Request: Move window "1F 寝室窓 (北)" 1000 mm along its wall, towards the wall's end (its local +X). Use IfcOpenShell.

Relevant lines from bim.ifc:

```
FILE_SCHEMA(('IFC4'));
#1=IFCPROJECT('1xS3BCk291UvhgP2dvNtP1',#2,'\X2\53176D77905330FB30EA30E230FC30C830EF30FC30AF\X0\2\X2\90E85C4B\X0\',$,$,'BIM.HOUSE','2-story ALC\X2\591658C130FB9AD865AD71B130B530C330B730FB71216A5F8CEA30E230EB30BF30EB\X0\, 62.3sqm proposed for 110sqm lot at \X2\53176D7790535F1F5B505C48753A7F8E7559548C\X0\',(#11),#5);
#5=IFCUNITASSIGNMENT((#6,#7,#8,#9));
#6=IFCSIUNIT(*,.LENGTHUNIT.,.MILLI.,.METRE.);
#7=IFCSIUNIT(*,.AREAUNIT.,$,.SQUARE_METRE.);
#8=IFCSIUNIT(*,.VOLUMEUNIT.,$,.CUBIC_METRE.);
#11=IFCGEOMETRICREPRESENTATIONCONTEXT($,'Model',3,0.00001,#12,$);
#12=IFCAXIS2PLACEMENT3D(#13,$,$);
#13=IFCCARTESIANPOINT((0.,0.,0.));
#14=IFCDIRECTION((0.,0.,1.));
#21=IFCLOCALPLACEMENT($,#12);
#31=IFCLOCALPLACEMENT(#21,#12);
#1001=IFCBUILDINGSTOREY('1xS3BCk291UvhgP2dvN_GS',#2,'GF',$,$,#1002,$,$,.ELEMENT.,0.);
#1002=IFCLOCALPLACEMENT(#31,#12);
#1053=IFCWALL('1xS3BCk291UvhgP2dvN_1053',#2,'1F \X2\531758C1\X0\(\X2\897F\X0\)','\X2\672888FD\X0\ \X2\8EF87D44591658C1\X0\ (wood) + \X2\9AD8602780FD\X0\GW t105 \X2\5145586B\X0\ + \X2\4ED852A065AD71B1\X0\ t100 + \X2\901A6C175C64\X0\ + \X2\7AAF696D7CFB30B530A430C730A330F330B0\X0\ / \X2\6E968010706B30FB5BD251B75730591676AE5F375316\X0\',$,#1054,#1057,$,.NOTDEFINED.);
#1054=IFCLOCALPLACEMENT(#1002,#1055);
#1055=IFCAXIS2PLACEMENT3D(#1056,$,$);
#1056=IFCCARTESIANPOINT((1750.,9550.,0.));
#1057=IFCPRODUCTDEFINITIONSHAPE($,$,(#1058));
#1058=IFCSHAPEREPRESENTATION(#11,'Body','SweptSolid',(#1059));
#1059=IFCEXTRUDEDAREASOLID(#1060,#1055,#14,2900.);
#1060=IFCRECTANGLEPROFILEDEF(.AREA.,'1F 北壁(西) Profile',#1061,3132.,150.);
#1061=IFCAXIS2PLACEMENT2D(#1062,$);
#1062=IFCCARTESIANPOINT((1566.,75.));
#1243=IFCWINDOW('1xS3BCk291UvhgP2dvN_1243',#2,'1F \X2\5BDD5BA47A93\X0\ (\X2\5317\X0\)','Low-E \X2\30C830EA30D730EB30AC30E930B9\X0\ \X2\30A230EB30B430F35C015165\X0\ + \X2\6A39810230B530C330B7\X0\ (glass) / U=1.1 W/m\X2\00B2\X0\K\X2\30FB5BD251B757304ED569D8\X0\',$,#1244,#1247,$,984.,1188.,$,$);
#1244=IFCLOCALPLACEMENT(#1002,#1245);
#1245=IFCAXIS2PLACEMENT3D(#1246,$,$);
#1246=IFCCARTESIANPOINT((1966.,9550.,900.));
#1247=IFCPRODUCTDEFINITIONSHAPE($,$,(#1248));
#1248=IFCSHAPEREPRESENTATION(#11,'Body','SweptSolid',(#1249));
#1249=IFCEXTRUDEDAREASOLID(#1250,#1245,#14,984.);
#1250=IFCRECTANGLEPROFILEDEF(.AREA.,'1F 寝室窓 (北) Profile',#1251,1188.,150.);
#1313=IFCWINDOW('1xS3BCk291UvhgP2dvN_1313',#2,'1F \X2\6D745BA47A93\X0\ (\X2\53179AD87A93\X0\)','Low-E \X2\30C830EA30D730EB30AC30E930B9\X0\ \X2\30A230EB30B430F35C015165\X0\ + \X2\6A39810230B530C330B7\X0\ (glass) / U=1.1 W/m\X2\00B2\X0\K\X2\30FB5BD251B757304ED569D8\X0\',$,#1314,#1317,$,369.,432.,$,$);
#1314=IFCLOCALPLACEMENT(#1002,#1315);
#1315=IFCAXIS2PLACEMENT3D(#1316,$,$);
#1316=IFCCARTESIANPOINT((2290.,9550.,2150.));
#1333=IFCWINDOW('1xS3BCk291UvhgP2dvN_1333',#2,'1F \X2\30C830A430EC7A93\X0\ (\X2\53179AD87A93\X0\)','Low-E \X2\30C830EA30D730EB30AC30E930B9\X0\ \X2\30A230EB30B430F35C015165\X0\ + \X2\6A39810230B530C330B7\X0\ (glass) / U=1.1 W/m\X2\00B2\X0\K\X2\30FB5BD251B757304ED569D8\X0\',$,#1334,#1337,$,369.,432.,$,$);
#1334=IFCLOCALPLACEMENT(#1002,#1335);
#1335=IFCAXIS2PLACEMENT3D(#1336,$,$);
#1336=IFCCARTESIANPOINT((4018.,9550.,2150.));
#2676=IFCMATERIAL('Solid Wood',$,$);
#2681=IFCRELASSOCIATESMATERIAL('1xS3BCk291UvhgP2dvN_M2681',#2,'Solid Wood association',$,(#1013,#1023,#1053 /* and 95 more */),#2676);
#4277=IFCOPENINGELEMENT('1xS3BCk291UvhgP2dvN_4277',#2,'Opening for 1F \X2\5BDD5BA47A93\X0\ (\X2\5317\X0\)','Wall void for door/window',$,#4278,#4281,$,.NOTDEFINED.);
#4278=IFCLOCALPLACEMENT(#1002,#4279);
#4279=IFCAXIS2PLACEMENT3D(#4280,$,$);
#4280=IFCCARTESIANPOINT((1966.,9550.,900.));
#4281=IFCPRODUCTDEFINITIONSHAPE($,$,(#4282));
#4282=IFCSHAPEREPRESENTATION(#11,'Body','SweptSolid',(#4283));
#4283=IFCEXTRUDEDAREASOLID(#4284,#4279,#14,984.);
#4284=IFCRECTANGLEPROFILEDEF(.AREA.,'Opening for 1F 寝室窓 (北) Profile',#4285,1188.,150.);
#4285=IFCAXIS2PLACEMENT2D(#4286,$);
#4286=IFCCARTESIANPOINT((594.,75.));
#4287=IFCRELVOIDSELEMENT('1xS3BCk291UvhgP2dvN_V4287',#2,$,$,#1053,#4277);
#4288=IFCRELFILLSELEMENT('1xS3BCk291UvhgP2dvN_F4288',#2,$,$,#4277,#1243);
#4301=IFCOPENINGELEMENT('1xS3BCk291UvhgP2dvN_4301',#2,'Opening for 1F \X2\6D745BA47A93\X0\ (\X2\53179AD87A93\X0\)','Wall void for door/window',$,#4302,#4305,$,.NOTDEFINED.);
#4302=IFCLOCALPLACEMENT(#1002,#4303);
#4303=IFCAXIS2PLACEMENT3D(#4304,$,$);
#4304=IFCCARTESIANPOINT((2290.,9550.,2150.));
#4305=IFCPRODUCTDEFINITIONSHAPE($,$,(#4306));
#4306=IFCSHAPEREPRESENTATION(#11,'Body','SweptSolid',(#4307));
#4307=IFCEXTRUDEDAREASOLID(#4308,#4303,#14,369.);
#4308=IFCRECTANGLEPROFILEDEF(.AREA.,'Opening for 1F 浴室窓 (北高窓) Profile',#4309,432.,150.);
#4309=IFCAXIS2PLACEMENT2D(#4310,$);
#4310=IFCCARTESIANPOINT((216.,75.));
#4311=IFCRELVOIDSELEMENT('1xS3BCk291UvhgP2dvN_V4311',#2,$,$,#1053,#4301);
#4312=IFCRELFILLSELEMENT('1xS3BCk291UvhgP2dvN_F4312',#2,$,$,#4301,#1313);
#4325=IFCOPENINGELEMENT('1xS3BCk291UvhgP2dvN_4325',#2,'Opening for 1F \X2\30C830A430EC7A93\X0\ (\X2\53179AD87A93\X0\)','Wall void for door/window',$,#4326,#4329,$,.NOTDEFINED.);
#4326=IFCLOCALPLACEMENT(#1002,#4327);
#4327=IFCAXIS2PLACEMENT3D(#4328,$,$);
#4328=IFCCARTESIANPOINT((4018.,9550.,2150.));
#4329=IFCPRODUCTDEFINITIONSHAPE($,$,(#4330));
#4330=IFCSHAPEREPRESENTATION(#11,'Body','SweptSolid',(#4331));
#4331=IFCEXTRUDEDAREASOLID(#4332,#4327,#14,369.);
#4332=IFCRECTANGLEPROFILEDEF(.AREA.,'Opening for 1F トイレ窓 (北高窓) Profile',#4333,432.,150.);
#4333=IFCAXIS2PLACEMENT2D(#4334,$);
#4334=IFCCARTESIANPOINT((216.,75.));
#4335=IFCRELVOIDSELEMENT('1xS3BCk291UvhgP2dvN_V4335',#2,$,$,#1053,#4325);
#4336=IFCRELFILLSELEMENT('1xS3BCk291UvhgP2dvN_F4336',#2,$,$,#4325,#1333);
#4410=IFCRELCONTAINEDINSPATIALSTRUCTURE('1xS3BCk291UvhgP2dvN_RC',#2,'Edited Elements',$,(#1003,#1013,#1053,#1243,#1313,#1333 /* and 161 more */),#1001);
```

```python
import ifcopenshell
import ifcopenshell.api.geometry
import ifcopenshell.util.placement

model = ifcopenshell.open("bim.ifc")

window = model.by_guid("1xS3BCk291UvhgP2dvN_1243")
opening = window.FillsVoids[0].RelatingOpeningElement
wall = opening.VoidsElements[0].RelatingBuildingElement

wall_matrix = ifcopenshell.util.placement.get_local_placement(wall.ObjectPlacement)
shift = wall_matrix[:3, 0] * 1000.0
before = ifcopenshell.util.placement.get_local_placement(window.ObjectPlacement)[:3, 3].copy()

# The window is not placed relative to its opening, so move both.
for product in (opening, window):
    matrix = ifcopenshell.util.placement.get_local_placement(product.ObjectPlacement)
    matrix[:3, 3] += shift
    ifcopenshell.api.geometry.edit_object_placement(model, product=product, matrix=matrix, is_si=False)

after = ifcopenshell.util.placement.get_local_placement(window.ObjectPlacement)[:3, 3]
print("window moved by", (after - before).round(3) + 0.0)

model.write("bim_updated.ifc")
```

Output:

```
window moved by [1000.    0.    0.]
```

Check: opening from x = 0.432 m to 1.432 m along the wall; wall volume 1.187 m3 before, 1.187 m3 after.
